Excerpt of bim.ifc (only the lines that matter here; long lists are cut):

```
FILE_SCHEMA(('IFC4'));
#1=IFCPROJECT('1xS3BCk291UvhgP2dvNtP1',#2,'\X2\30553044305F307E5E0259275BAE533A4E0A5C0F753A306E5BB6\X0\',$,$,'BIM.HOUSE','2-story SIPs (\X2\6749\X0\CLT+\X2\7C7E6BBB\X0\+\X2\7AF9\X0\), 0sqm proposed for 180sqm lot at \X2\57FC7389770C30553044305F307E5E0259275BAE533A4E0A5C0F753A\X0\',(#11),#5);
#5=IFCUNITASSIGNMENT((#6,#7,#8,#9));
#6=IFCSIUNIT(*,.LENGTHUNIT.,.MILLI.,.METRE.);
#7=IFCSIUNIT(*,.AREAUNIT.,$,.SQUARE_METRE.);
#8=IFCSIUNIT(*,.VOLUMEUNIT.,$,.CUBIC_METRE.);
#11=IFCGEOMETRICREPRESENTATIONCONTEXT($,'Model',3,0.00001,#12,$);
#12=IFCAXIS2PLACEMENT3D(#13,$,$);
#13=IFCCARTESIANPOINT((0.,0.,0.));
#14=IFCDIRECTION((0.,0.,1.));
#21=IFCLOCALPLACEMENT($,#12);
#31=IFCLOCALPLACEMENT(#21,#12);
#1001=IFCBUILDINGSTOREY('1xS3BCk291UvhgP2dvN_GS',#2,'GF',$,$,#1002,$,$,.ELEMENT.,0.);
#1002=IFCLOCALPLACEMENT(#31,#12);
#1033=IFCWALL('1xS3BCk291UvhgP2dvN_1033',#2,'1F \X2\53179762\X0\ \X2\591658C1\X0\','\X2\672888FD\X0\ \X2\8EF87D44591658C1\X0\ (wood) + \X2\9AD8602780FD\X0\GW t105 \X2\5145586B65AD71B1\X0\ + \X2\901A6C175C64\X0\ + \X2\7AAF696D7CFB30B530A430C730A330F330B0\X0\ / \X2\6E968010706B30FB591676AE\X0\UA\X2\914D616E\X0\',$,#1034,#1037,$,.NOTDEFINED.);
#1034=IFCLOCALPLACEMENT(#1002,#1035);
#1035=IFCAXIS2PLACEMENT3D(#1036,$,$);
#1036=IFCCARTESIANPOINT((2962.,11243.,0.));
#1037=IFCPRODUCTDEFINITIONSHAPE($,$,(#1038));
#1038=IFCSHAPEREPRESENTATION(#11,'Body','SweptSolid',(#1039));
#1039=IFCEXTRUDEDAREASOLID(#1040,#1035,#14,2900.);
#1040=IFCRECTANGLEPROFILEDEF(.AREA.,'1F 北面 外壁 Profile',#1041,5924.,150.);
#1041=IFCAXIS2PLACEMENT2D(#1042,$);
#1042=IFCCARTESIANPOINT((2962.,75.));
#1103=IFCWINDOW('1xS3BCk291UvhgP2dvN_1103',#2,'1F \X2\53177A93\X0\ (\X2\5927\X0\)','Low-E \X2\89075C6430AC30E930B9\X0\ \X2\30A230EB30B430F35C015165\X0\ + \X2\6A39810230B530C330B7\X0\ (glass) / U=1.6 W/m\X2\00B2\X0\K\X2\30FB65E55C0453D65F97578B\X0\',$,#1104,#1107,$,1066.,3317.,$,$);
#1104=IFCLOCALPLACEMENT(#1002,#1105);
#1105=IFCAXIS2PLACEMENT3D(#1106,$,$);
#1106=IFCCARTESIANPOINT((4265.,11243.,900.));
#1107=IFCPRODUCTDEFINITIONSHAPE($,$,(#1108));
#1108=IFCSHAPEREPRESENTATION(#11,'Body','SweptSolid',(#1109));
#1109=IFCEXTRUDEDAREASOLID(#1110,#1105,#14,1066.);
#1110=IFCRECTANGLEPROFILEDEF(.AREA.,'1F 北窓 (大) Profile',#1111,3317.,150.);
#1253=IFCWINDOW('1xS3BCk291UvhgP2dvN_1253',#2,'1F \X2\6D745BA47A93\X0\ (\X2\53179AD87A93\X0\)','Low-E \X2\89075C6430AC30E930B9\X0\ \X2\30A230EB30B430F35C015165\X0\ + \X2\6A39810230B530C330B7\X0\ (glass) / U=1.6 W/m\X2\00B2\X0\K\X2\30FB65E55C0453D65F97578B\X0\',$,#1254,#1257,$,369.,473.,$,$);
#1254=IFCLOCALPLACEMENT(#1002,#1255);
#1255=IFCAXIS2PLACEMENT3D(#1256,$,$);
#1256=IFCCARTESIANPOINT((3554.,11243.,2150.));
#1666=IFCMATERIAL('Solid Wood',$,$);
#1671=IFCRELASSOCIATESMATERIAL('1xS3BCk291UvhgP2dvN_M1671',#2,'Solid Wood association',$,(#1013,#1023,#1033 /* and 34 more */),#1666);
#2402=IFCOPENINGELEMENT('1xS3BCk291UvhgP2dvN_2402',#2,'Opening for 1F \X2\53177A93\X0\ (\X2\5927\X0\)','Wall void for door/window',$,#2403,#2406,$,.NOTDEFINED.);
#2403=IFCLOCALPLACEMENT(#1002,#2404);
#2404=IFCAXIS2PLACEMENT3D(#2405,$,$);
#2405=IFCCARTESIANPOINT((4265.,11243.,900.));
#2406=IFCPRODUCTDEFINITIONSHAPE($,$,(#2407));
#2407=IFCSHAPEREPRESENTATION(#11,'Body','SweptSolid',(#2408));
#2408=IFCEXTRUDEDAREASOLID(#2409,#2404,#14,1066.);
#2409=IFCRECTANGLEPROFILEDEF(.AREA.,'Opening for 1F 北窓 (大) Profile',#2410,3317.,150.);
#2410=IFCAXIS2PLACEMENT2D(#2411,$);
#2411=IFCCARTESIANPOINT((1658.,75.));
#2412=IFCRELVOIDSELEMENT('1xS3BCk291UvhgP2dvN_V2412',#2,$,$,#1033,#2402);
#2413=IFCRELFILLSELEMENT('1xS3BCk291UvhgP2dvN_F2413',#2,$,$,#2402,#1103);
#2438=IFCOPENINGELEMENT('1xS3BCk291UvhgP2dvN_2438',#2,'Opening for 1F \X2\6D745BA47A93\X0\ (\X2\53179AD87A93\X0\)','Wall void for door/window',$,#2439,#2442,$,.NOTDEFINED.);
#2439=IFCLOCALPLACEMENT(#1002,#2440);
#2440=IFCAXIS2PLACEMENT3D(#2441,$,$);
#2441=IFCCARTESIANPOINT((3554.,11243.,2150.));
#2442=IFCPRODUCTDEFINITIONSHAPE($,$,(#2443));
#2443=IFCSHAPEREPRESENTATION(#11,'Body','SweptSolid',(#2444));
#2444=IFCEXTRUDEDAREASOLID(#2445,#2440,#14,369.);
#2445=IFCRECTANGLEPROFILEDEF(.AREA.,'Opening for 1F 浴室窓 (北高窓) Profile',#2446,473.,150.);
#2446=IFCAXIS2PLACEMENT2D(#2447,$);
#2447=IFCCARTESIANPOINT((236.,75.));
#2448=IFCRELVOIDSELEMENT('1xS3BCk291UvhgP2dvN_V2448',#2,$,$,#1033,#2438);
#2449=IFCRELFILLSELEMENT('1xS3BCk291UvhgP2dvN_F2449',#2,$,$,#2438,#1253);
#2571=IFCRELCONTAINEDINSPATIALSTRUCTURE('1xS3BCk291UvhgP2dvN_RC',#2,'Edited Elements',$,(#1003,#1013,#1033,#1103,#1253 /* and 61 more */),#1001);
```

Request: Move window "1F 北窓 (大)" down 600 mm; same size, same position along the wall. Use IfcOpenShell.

```python
import numpy as np
import ifcopenshell
import ifcopenshell.api.geometry
import ifcopenshell.util.placement
import ifcopenshell.util.unit

model = ifcopenshell.open("bim.ifc")
unit_scale = ifcopenshell.util.unit.calculate_unit_scale(model)

window = model.by_guid("1xS3BCk291UvhgP2dvN_1103")
opening = window.FillsVoids[0].RelatingOpeningElement
dz = -600.0

shift = np.array([0.0, 0.0, dz])
# The window is not placed relative to its opening, so move both.
for product in (opening, window):
    matrix = ifcopenshell.util.placement.get_local_placement(product.ObjectPlacement)
    matrix[:3, 3] += shift
    ifcopenshell.api.geometry.edit_object_placement(model, product=product, matrix=matrix, is_si=False)

print(f"moved by {dz * unit_scale:+.3f} m")

model.write("bim_edited.ifc")
```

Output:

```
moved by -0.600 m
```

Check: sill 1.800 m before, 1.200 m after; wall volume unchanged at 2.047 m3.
